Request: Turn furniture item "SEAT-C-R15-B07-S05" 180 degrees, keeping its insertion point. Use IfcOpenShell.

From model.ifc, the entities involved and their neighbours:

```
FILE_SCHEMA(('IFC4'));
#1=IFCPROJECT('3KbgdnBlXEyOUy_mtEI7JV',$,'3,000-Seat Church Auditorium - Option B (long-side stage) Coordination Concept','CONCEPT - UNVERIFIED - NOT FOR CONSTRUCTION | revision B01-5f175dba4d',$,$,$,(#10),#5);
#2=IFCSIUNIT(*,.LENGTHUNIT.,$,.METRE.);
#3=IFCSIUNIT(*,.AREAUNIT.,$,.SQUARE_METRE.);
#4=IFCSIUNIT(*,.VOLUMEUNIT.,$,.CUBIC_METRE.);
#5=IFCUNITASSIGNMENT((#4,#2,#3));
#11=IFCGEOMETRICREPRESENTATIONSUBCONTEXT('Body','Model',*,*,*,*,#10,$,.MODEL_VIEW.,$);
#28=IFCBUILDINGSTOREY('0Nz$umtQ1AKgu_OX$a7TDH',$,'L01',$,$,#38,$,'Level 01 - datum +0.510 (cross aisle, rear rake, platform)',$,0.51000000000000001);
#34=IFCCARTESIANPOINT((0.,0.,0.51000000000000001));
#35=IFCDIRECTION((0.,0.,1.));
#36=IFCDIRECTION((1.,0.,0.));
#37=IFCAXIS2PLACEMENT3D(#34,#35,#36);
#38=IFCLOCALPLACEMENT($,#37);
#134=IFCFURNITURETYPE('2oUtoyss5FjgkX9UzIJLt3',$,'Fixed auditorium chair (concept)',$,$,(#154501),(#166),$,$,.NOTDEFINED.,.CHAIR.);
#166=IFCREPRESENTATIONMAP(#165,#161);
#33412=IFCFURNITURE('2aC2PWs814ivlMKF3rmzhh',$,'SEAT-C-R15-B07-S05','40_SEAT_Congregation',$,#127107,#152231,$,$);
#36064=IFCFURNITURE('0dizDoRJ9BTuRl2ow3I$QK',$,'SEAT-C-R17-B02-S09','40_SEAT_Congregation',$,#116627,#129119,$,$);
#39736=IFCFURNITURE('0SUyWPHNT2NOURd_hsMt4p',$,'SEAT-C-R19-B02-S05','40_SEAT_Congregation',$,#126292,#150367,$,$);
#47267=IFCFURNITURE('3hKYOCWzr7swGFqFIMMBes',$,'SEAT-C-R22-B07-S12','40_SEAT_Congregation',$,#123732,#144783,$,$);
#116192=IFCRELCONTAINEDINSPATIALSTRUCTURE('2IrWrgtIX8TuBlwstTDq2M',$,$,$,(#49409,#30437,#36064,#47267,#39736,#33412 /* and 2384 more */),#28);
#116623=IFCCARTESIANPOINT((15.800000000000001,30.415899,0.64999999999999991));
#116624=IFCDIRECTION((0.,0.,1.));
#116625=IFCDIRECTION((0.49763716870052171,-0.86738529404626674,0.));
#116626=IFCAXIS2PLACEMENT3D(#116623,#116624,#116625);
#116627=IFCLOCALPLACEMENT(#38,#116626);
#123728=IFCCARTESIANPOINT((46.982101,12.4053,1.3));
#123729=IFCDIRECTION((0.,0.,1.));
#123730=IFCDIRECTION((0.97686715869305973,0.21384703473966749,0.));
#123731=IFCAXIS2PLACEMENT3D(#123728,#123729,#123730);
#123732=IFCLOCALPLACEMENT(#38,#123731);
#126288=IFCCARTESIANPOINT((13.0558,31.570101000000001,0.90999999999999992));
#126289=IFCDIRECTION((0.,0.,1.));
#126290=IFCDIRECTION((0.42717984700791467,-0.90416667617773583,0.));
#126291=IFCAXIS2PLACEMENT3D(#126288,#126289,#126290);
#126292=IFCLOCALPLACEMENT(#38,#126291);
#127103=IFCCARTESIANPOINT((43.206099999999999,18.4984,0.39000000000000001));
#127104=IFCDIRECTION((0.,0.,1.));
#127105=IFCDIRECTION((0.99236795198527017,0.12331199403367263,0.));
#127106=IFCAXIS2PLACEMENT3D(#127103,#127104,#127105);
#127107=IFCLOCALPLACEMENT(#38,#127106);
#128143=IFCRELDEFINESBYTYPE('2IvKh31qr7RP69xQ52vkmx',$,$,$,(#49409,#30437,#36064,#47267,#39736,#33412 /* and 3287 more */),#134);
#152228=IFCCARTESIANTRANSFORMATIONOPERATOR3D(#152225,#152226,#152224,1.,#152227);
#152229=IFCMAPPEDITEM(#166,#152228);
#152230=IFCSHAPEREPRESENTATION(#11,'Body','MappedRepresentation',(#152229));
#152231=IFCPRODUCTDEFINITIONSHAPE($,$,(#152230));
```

```python
import ifcopenshell
import ifcopenshell.api.geometry
import ifcopenshell.util.placement

model = ifcopenshell.open("model.ifc")

item = model.by_guid("2aC2PWs814ivlMKF3rmzhh")
matrix = ifcopenshell.util.placement.get_local_placement(item.ObjectPlacement)
matrix = matrix @ ifcopenshell.util.placement.rotation(180, "Z")
ifcopenshell.api.geometry.edit_object_placement(model, product=item, matrix=matrix, is_si=False)

print(ifcopenshell.util.placement.get_local_placement(item.ObjectPlacement).round(3) + 0.0)

model.write("model_v2.ifc")
```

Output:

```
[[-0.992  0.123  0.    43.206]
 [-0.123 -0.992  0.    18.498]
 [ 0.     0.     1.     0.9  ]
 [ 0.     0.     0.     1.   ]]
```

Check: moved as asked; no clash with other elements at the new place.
